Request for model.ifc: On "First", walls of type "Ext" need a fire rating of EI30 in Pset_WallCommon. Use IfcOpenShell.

First a look at what the model holds.

```python
import ifcopenshell
import ifcopenshell.util.element

model = ifcopenshell.open("model.ifc")
print(model.schema)
storey = next(s for s in model.by_type("IfcBuildingStorey") if s.Name == "First")
walls = [e for e in ifcopenshell.util.element.get_decomposition(storey) if e.is_a("IfcWall")]
seen = {}
for e in walls:
    element_type = ifcopenshell.util.element.get_type(e)
    key = (element_type.Name if element_type != e and element_type else None, ifcopenshell.util.element.get_pset(e, "Pset_WallCommon", "FireRating"))
    seen[key] = seen.get(key, 0) + 1
for (name, value), count in sorted(seen.items(), key=str):
    print(count, "x", name, "|", value)
```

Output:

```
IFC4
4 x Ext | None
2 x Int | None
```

```python
import ifcopenshell
import ifcopenshell.api.pset
import ifcopenshell.util.element

model = ifcopenshell.open("model.ifc")

storey = next(s for s in model.by_type("IfcBuildingStorey") if s.Name == "First")
walls = [e for e in ifcopenshell.util.element.get_decomposition(storey) if e.is_a("IfcWall")]

count = 0
for e in walls:
    element_type = ifcopenshell.util.element.get_type(e)
    if element_type in (None, e) or element_type.Name != "Ext":
        continue
    # add_pset returns the element's existing set when there is one.
    pset = ifcopenshell.api.pset.add_pset(model, product=e, name="Pset_WallCommon")
    ifcopenshell.api.pset.edit_pset(model, pset=pset, properties={"FireRating": "EI30"})
    count += 1

print(count, "walls updated")

model.write("model_rev.ifc")
```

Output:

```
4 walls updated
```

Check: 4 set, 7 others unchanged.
